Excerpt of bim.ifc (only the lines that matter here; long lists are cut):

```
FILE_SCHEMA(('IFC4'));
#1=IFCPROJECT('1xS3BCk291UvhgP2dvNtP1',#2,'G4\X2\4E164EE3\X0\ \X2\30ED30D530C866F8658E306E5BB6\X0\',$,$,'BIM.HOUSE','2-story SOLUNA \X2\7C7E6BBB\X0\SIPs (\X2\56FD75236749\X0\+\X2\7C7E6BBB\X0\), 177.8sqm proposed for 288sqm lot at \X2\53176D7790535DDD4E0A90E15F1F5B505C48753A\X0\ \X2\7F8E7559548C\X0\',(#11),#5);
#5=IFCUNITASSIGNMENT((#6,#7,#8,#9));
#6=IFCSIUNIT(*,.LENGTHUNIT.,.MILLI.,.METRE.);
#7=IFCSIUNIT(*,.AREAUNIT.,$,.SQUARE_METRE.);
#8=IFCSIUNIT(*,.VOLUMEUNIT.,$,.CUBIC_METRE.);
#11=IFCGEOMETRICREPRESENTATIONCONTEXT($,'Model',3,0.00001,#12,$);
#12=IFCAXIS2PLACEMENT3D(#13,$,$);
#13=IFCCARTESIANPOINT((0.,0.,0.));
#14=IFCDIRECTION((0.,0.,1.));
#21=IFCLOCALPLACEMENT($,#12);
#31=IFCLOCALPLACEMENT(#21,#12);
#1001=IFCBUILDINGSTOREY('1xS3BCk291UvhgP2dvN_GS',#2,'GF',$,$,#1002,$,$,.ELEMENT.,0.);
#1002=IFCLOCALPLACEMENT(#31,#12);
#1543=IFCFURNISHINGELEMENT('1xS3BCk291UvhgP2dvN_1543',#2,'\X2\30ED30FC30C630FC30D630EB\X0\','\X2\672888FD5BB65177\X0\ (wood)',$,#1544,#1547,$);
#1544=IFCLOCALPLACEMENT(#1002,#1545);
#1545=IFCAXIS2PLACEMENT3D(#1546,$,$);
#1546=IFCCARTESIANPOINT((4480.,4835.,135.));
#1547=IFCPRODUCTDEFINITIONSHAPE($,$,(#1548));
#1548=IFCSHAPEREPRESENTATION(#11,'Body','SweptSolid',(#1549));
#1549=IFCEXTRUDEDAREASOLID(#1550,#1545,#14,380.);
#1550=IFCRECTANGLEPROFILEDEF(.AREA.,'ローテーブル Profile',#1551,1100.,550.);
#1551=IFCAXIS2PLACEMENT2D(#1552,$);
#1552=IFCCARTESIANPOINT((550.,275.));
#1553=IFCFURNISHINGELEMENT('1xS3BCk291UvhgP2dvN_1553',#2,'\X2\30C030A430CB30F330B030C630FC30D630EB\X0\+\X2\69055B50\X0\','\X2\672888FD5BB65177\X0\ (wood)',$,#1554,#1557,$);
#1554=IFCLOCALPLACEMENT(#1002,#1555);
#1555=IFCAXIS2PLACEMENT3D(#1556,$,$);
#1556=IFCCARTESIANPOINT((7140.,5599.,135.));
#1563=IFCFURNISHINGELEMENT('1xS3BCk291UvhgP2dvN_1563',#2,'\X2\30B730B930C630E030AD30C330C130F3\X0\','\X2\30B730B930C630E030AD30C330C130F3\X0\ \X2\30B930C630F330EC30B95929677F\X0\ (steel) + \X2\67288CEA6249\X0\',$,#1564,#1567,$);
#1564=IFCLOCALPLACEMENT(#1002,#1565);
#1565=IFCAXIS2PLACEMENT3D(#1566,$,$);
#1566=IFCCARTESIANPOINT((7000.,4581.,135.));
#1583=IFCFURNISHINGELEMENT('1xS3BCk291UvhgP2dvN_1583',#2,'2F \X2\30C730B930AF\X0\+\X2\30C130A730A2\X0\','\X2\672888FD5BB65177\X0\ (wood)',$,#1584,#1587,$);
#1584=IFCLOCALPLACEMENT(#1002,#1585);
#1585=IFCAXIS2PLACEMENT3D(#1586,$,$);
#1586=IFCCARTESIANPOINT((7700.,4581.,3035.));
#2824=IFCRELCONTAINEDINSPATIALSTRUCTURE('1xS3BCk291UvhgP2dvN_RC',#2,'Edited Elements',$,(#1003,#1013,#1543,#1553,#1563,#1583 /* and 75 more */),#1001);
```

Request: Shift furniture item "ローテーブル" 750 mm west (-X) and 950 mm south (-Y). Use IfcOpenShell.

```python
import ifcopenshell
import ifcopenshell.api.geometry
import ifcopenshell.util.placement
import ifcopenshell.util.unit

model = ifcopenshell.open("bim.ifc")
unit_scale = ifcopenshell.util.unit.calculate_unit_scale(model)

item = model.by_id(1543)
matrix = ifcopenshell.util.placement.get_local_placement(item.ObjectPlacement)
matrix[0, 3] -= 0.75 / unit_scale
matrix[1, 3] -= 0.95 / unit_scale
ifcopenshell.api.geometry.edit_object_placement(model, product=item, matrix=matrix, is_si=False)

print(ifcopenshell.util.placement.get_local_placement(item.ObjectPlacement).round(3) + 0.0)

model.write("bim_updated.ifc")
```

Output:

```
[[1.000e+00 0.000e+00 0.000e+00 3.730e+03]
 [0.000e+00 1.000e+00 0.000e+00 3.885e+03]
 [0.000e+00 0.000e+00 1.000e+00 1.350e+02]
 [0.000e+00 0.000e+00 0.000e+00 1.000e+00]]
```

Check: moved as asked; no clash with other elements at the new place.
